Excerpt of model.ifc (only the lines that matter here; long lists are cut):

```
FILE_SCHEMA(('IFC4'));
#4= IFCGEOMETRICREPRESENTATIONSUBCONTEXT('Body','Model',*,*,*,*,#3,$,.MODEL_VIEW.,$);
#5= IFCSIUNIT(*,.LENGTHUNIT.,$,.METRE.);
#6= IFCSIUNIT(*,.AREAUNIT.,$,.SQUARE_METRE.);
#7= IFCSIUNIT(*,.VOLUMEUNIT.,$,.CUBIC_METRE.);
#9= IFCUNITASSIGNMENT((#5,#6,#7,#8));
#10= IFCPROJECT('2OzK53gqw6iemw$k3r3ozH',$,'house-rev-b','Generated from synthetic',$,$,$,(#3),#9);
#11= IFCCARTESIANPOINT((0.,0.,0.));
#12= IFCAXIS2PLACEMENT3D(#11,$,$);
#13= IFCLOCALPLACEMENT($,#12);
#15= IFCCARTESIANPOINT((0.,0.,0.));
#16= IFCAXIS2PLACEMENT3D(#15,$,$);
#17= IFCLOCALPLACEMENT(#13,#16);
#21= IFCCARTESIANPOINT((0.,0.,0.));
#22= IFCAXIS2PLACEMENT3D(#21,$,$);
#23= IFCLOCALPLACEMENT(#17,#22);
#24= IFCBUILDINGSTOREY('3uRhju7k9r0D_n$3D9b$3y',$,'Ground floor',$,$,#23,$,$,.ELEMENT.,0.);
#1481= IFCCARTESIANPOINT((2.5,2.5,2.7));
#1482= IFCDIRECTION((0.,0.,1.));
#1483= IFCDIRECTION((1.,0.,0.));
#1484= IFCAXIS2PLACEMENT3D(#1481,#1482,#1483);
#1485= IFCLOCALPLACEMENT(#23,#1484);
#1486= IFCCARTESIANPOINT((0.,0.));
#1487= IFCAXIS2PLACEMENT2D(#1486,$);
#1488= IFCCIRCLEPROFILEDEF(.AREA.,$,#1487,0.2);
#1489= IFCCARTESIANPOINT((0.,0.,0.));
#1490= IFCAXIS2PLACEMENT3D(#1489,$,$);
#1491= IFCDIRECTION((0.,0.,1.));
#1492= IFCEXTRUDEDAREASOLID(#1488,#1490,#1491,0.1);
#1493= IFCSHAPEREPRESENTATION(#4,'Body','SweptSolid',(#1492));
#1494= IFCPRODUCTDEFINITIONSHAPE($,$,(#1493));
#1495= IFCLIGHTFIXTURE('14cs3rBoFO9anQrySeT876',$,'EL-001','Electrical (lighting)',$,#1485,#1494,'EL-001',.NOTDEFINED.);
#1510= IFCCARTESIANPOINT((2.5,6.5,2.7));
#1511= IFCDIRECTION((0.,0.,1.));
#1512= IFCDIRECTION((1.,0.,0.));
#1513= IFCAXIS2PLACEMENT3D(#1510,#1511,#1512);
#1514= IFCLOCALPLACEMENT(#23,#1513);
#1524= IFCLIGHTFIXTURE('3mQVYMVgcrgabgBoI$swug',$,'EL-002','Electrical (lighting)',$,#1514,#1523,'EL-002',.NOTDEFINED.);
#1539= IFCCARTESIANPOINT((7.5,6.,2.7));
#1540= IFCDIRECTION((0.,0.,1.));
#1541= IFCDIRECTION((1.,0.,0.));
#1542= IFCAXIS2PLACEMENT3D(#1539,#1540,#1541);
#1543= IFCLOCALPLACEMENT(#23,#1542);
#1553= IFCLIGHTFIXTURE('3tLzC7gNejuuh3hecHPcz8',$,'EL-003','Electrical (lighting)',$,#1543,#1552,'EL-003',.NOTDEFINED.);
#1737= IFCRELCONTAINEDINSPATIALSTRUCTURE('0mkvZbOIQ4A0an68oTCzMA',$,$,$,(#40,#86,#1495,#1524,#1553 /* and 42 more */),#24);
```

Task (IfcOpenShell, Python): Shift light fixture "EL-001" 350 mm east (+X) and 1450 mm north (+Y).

```python
import ifcopenshell
import ifcopenshell.api.geometry
import ifcopenshell.util.placement
import ifcopenshell.util.unit

model = ifcopenshell.open("model.ifc")
unit_scale = ifcopenshell.util.unit.calculate_unit_scale(model)

item = model.by_guid("14cs3rBoFO9anQrySeT876")
matrix = ifcopenshell.util.placement.get_local_placement(item.ObjectPlacement)
matrix[0, 3] += 0.35 / unit_scale
matrix[1, 3] += 1.45 / unit_scale
ifcopenshell.api.geometry.edit_object_placement(model, product=item, matrix=matrix, is_si=False)

print(ifcopenshell.util.placement.get_local_placement(item.ObjectPlacement).round(3) + 0.0)

model.write("model-out.ifc")
```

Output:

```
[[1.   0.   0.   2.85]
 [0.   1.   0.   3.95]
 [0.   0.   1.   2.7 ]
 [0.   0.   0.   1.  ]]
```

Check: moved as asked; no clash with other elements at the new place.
